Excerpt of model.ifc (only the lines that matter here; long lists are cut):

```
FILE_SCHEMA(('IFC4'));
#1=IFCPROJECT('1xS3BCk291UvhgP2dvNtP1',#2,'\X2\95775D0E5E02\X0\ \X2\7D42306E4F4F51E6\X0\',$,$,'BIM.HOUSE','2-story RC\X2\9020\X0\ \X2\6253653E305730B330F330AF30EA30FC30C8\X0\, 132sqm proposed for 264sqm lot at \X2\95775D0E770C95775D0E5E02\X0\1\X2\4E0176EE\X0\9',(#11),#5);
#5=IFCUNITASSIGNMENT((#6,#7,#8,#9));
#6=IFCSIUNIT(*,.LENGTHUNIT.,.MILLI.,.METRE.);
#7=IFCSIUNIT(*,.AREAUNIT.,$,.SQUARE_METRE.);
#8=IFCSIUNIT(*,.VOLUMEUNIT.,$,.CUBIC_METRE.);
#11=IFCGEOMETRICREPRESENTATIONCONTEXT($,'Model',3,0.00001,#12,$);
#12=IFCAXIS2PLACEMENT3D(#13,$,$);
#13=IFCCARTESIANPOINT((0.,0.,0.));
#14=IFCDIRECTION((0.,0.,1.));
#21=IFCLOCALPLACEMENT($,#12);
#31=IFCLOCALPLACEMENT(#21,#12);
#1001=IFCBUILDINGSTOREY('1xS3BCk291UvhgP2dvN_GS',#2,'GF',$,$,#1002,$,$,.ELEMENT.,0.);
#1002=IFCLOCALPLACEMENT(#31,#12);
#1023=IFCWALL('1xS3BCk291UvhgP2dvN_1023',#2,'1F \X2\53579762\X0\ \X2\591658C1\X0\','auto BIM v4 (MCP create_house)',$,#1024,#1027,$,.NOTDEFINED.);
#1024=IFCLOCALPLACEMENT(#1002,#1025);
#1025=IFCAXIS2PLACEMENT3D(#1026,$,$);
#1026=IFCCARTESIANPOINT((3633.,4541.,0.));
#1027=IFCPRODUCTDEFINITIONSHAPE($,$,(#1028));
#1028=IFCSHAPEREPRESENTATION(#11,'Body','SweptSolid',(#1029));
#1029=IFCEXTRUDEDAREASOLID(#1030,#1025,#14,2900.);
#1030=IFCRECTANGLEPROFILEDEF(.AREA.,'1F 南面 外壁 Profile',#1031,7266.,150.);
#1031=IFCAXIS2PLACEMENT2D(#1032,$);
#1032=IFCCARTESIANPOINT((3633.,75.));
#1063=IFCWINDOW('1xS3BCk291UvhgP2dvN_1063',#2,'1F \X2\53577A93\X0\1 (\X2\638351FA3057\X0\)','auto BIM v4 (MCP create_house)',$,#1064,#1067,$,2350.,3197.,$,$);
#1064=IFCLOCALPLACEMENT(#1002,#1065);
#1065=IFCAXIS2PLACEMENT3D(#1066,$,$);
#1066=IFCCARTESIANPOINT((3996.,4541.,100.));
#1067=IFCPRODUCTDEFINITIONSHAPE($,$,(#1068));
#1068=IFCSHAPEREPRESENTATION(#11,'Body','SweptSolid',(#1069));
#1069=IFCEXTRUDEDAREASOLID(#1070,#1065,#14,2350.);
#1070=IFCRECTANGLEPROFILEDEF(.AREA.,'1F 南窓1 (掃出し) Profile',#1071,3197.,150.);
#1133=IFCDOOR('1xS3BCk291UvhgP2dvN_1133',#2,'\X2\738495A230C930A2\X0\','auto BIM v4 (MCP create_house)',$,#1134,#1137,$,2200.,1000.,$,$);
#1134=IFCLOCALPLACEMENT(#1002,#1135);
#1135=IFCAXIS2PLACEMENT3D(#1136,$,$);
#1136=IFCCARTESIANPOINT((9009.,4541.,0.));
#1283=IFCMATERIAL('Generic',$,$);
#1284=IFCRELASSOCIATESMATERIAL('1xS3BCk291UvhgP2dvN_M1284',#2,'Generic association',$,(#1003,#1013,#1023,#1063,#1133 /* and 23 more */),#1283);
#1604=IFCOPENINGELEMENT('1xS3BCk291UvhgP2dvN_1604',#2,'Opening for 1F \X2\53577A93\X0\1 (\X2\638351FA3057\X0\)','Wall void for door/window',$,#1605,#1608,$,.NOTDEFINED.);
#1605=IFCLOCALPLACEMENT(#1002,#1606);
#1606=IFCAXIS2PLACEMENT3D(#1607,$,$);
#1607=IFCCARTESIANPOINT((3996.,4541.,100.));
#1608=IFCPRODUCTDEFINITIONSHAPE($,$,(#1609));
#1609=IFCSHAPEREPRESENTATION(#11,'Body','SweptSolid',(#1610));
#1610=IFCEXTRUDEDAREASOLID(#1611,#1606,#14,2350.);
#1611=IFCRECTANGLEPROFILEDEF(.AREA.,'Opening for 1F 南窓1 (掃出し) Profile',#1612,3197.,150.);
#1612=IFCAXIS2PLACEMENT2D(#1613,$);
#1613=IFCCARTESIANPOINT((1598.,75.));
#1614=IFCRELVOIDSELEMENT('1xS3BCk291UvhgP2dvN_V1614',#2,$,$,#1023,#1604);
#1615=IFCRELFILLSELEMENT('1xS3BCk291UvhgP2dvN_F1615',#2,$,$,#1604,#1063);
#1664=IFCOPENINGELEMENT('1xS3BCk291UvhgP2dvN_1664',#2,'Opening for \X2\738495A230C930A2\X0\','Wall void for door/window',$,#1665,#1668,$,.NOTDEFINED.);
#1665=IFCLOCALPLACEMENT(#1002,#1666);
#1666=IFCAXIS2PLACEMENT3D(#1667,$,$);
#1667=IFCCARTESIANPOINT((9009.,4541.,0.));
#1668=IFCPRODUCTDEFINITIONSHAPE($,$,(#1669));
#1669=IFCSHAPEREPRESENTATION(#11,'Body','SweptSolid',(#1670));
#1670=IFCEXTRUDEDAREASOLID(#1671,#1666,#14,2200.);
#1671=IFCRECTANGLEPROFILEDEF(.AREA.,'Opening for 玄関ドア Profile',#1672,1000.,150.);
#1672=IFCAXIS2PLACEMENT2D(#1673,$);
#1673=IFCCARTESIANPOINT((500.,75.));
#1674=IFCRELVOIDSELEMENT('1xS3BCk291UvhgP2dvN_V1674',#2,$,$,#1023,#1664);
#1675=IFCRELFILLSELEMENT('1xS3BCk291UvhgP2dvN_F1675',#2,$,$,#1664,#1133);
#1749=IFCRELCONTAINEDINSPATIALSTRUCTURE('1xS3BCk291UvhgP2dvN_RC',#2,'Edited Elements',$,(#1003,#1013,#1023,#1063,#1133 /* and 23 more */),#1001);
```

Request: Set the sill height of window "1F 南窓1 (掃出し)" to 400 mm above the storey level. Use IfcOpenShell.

```python
import numpy as np
import ifcopenshell
import ifcopenshell.api.geometry
import ifcopenshell.geom
import ifcopenshell.util.element
import ifcopenshell.util.placement
import ifcopenshell.util.shape
import ifcopenshell.util.unit

model = ifcopenshell.open("model.ifc")
unit_scale = ifcopenshell.util.unit.calculate_unit_scale(model)

window = model.by_guid("1xS3BCk291UvhgP2dvN_1063")
opening = window.FillsVoids[0].RelatingOpeningElement
storey = ifcopenshell.util.element.get_container(window, ifc_class="IfcBuildingStorey")
level = ifcopenshell.util.placement.get_local_placement(storey.ObjectPlacement)[2, 3]

# The opening's origin need not be at the sill, so measure its lowest point.
shape = ifcopenshell.geom.create_shape(ifcopenshell.geom.settings(), opening)
bottom = ifcopenshell.util.shape.get_shape_bottom_elevation(shape, shape.geometry) / unit_scale
dz = level + 400.0 - bottom

shift = np.array([0.0, 0.0, dz])
# The window is not placed relative to its opening, so move both.
for product in (opening, window):
    matrix = ifcopenshell.util.placement.get_local_placement(product.ObjectPlacement)
    matrix[:3, 3] += shift
    ifcopenshell.api.geometry.edit_object_placement(model, product=product, matrix=matrix, is_si=False)

print(f"moved by {dz * unit_scale:+.3f} m")

model.write("model_edited.ifc")
```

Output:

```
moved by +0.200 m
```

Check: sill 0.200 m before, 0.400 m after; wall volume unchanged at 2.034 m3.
